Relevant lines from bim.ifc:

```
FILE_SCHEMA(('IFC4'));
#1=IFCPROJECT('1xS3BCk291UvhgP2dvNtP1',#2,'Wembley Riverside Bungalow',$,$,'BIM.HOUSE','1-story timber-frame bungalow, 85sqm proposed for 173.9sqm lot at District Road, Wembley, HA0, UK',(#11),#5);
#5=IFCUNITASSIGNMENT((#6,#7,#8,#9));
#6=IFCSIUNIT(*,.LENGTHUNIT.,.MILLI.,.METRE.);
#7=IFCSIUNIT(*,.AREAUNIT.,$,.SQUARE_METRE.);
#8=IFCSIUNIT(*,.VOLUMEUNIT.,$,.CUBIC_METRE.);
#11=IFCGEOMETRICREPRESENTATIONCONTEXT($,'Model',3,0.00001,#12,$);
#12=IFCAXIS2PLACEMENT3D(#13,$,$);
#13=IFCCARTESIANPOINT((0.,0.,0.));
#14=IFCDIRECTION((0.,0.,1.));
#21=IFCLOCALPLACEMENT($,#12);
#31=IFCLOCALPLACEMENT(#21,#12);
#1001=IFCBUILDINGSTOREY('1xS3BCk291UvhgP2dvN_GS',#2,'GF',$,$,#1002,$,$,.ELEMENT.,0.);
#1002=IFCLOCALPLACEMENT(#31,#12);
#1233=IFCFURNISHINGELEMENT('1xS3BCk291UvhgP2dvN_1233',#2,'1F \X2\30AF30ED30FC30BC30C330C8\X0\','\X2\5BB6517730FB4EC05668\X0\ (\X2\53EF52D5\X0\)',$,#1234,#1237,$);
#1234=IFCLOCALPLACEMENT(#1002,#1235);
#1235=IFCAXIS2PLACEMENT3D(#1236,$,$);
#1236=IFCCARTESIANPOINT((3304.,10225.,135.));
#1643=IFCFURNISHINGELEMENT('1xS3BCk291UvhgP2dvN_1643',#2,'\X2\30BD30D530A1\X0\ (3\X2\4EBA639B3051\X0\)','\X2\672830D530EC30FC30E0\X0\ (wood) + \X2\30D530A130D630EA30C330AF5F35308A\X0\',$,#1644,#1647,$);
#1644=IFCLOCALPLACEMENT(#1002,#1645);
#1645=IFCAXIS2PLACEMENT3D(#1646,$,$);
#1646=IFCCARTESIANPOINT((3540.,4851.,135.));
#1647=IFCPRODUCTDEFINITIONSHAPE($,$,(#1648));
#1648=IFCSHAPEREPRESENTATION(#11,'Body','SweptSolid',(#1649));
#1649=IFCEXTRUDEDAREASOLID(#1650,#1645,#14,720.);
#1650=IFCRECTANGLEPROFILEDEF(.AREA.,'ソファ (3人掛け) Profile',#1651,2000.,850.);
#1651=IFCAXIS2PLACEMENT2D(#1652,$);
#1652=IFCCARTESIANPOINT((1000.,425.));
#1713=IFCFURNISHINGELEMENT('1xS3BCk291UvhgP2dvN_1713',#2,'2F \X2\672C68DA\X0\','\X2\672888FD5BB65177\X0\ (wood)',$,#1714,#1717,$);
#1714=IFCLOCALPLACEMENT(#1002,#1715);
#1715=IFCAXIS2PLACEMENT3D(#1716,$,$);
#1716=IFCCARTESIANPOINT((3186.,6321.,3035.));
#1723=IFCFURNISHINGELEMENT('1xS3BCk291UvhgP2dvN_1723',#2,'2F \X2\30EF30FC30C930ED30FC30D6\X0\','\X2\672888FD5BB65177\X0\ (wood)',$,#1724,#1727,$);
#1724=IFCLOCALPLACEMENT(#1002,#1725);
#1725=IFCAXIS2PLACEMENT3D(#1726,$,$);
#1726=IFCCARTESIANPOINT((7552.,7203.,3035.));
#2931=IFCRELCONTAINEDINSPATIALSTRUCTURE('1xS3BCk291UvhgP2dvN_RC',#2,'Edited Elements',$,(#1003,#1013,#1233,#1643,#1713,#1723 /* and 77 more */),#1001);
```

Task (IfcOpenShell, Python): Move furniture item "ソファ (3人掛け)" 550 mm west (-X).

```python
import ifcopenshell
import ifcopenshell.api.geometry
import ifcopenshell.util.placement

model = ifcopenshell.open("bim.ifc")

item = model.by_guid("1xS3BCk291UvhgP2dvN_1643")
matrix = ifcopenshell.util.placement.get_local_placement(item.ObjectPlacement)
matrix[0, 3] -= 550.0
ifcopenshell.api.geometry.edit_object_placement(model, product=item, matrix=matrix, is_si=False)

print(ifcopenshell.util.placement.get_local_placement(item.ObjectPlacement).round(3) + 0.0)

model.write("bim_updated.ifc")
```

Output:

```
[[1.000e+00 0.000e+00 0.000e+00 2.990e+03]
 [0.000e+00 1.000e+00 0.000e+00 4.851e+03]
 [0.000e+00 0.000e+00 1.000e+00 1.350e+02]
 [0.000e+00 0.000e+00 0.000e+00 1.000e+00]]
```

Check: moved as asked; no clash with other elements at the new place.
